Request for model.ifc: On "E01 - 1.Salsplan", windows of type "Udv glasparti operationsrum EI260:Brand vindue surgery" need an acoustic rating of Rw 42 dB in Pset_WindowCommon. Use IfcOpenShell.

First a look at what the model holds.

```python
import ifcopenshell
import ifcopenshell.util.element

model = ifcopenshell.open("model.ifc")
print(model.schema)
storey = next(s for s in model.by_type("IfcBuildingStorey") if s.Name == "E01 - 1.Salsplan")
windows = [e for e in ifcopenshell.util.element.get_decomposition(storey) if e.is_a("IfcWindow")]
seen = {}
for e in windows:
    element_type = ifcopenshell.util.element.get_type(e)
    key = (element_type.Name if element_type != e and element_type else None, ifcopenshell.util.element.get_pset(e, "Pset_WindowCommon", "AcousticRating"))
    seen[key] = seen.get(key, 0) + 1
for (name, value), count in sorted(seen.items(), key=str):
    print(count, "x", name, "|", value)
```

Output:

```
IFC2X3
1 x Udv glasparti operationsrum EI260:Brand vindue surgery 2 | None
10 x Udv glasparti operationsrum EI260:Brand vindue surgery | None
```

```python
import ifcopenshell
import ifcopenshell.api.pset
import ifcopenshell.util.element

model = ifcopenshell.open("model.ifc")

storey = next(s for s in model.by_type("IfcBuildingStorey") if s.Name == "E01 - 1.Salsplan")
windows = [e for e in ifcopenshell.util.element.get_decomposition(storey) if e.is_a("IfcWindow")]

count = 0
for e in windows:
    element_type = ifcopenshell.util.element.get_type(e)
    if element_type in (None, e) or element_type.Name != "Udv glasparti operationsrum EI260:Brand vindue surgery":
        continue
    # add_pset returns the element's existing set when there is one.
    pset = ifcopenshell.api.pset.add_pset(model, product=e, name="Pset_WindowCommon")
    ifcopenshell.api.pset.edit_pset(model, pset=pset, properties={"AcousticRating": "Rw 42 dB"})
    count += 1

print(count, "windows updated")

model.write("model-out.ifc")
```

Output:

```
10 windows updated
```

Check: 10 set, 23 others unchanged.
